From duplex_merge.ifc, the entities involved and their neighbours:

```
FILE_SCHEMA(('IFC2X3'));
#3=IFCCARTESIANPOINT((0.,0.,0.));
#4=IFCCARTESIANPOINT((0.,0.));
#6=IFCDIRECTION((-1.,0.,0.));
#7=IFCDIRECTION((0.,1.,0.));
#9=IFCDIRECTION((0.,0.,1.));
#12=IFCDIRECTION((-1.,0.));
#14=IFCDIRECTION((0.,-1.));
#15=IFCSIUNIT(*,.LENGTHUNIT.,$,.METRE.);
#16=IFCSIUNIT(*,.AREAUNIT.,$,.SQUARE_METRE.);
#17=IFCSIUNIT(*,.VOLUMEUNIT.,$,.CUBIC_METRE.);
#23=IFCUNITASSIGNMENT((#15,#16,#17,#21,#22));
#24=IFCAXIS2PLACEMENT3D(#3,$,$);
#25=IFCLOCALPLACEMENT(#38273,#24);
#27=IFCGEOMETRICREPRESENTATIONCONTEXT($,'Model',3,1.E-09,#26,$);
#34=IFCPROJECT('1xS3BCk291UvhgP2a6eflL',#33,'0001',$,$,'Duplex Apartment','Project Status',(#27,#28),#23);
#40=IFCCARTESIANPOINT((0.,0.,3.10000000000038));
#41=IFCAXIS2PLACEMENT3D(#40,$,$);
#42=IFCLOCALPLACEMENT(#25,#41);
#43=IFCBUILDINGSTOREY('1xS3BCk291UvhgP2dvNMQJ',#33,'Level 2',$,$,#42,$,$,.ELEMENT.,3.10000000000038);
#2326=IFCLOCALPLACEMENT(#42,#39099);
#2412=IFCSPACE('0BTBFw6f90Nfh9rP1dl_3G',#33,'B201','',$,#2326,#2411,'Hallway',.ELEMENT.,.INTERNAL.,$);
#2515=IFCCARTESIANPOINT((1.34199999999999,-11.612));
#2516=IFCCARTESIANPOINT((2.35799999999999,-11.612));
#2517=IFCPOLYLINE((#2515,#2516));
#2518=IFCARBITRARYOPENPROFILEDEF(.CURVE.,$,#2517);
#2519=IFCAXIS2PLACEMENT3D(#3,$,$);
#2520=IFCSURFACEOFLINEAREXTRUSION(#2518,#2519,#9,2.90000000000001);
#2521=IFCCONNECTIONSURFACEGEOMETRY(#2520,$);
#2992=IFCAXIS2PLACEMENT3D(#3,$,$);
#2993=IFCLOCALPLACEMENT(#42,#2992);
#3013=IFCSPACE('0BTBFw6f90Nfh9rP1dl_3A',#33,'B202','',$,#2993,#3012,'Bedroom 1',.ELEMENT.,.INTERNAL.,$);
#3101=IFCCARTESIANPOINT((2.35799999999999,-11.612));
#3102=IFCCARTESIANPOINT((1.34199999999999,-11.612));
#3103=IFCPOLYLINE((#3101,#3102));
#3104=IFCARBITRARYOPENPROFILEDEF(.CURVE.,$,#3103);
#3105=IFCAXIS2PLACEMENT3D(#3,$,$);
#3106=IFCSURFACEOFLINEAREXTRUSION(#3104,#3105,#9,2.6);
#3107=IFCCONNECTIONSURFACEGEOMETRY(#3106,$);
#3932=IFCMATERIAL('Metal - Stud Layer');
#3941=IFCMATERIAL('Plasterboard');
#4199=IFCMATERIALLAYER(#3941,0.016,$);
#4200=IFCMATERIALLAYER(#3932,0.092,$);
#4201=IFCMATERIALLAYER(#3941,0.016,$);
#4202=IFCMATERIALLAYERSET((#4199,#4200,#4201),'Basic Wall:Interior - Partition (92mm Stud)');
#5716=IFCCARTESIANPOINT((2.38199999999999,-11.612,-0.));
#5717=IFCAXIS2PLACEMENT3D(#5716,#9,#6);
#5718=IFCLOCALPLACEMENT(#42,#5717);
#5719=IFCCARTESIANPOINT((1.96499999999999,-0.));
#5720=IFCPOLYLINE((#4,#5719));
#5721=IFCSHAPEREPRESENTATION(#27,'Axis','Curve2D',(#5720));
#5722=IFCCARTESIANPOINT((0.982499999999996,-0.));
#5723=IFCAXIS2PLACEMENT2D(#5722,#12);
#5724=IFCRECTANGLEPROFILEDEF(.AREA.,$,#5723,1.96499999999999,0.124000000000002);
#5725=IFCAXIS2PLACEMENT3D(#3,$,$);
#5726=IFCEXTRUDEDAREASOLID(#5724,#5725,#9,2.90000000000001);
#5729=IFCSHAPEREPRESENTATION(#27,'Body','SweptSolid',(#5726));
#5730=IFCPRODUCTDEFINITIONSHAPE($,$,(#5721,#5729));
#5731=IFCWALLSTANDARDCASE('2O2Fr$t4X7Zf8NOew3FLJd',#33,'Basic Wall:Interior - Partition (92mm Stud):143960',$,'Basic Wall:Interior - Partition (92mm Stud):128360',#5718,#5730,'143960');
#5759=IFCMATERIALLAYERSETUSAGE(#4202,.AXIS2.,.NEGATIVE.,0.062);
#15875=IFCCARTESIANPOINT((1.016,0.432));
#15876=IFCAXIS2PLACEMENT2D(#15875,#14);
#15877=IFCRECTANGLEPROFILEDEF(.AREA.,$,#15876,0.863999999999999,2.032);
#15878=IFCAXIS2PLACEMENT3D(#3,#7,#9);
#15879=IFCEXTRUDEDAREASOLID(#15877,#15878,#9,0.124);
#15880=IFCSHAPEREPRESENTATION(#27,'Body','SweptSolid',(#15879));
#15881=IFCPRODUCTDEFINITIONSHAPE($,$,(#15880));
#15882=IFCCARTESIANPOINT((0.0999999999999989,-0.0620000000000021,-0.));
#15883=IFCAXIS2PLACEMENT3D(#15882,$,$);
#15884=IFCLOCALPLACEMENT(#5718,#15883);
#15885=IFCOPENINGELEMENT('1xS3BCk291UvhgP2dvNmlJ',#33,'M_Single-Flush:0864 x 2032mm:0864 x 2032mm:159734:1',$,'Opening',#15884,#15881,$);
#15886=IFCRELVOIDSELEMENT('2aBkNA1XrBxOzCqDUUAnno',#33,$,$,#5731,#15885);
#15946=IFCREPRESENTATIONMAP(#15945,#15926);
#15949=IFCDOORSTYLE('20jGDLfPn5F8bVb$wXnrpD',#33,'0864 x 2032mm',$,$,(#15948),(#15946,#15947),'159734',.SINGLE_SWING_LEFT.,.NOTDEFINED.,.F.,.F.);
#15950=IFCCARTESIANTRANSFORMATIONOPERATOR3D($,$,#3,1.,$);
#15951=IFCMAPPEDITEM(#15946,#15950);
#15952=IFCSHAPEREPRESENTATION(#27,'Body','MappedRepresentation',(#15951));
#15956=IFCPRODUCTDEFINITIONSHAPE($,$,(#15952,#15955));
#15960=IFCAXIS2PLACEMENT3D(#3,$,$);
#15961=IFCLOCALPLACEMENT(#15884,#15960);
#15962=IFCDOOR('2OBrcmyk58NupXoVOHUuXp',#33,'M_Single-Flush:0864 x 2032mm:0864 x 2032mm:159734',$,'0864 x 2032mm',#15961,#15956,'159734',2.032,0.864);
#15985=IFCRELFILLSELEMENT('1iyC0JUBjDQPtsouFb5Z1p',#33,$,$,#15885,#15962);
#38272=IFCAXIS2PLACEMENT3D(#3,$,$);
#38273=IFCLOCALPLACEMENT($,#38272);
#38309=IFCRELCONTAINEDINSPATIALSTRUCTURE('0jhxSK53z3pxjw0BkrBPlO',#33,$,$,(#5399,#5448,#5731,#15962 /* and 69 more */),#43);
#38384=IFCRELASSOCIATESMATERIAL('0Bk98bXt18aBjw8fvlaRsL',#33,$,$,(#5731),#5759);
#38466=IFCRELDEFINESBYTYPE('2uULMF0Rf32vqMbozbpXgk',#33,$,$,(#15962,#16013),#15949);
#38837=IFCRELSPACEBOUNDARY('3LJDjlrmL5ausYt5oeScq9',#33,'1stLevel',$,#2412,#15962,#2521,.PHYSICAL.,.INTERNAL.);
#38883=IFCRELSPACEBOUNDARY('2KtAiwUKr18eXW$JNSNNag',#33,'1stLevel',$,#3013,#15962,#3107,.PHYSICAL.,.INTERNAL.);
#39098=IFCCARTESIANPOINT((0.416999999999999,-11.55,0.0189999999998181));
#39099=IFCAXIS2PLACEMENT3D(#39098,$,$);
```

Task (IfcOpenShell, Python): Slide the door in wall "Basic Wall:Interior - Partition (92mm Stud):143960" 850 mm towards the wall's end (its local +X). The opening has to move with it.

```python
import numpy as np
import ifcopenshell
import ifcopenshell.api.geometry
import ifcopenshell.util.placement
import ifcopenshell.util.unit

model = ifcopenshell.open("duplex_merge.ifc")
unit_scale = ifcopenshell.util.unit.calculate_unit_scale(model)

door = model.by_guid("2OBrcmyk58NupXoVOHUuXp")
opening = door.FillsVoids[0].RelatingOpeningElement
wall = opening.VoidsElements[0].RelatingBuildingElement

wall_matrix = ifcopenshell.util.placement.get_local_placement(wall.ObjectPlacement)
shift = wall_matrix[:3, 0] * 0.85 / unit_scale
before = ifcopenshell.util.placement.get_local_placement(door.ObjectPlacement)[:3, 3].copy()

# The door is placed relative to its opening, so it follows when the opening moves.
matrix = ifcopenshell.util.placement.get_local_placement(opening.ObjectPlacement)
matrix[:3, 3] += shift
ifcopenshell.api.geometry.edit_object_placement(
    model, product=opening, matrix=matrix, is_si=False, should_transform_children=True
)

# Space boundary surfaces are stored in each space's coordinates; move them too.
for rel in door.ProvidesBoundaries:
    if not rel.ConnectionGeometry:
        continue
    surface = rel.ConnectionGeometry.SurfaceOnRelatingElement
    space_matrix = ifcopenshell.util.placement.get_local_placement(rel.RelatingSpace.ObjectPlacement)
    point = np.array(surface.Position.Location.Coordinates) + space_matrix[:3, :3].T @ shift
    surface.Position = model.createIfcAxis2Placement3D(
        model.createIfcCartesianPoint(point.tolist()), surface.Position.Axis, surface.Position.RefDirection
    )

after = ifcopenshell.util.placement.get_local_placement(door.ObjectPlacement)[:3, 3]
print("door moved by", (after - before).round(3) + 0.0)

model.write("duplex_merge_v2.ifc")
```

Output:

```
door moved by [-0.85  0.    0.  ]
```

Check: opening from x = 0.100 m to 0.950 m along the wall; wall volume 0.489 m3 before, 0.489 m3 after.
